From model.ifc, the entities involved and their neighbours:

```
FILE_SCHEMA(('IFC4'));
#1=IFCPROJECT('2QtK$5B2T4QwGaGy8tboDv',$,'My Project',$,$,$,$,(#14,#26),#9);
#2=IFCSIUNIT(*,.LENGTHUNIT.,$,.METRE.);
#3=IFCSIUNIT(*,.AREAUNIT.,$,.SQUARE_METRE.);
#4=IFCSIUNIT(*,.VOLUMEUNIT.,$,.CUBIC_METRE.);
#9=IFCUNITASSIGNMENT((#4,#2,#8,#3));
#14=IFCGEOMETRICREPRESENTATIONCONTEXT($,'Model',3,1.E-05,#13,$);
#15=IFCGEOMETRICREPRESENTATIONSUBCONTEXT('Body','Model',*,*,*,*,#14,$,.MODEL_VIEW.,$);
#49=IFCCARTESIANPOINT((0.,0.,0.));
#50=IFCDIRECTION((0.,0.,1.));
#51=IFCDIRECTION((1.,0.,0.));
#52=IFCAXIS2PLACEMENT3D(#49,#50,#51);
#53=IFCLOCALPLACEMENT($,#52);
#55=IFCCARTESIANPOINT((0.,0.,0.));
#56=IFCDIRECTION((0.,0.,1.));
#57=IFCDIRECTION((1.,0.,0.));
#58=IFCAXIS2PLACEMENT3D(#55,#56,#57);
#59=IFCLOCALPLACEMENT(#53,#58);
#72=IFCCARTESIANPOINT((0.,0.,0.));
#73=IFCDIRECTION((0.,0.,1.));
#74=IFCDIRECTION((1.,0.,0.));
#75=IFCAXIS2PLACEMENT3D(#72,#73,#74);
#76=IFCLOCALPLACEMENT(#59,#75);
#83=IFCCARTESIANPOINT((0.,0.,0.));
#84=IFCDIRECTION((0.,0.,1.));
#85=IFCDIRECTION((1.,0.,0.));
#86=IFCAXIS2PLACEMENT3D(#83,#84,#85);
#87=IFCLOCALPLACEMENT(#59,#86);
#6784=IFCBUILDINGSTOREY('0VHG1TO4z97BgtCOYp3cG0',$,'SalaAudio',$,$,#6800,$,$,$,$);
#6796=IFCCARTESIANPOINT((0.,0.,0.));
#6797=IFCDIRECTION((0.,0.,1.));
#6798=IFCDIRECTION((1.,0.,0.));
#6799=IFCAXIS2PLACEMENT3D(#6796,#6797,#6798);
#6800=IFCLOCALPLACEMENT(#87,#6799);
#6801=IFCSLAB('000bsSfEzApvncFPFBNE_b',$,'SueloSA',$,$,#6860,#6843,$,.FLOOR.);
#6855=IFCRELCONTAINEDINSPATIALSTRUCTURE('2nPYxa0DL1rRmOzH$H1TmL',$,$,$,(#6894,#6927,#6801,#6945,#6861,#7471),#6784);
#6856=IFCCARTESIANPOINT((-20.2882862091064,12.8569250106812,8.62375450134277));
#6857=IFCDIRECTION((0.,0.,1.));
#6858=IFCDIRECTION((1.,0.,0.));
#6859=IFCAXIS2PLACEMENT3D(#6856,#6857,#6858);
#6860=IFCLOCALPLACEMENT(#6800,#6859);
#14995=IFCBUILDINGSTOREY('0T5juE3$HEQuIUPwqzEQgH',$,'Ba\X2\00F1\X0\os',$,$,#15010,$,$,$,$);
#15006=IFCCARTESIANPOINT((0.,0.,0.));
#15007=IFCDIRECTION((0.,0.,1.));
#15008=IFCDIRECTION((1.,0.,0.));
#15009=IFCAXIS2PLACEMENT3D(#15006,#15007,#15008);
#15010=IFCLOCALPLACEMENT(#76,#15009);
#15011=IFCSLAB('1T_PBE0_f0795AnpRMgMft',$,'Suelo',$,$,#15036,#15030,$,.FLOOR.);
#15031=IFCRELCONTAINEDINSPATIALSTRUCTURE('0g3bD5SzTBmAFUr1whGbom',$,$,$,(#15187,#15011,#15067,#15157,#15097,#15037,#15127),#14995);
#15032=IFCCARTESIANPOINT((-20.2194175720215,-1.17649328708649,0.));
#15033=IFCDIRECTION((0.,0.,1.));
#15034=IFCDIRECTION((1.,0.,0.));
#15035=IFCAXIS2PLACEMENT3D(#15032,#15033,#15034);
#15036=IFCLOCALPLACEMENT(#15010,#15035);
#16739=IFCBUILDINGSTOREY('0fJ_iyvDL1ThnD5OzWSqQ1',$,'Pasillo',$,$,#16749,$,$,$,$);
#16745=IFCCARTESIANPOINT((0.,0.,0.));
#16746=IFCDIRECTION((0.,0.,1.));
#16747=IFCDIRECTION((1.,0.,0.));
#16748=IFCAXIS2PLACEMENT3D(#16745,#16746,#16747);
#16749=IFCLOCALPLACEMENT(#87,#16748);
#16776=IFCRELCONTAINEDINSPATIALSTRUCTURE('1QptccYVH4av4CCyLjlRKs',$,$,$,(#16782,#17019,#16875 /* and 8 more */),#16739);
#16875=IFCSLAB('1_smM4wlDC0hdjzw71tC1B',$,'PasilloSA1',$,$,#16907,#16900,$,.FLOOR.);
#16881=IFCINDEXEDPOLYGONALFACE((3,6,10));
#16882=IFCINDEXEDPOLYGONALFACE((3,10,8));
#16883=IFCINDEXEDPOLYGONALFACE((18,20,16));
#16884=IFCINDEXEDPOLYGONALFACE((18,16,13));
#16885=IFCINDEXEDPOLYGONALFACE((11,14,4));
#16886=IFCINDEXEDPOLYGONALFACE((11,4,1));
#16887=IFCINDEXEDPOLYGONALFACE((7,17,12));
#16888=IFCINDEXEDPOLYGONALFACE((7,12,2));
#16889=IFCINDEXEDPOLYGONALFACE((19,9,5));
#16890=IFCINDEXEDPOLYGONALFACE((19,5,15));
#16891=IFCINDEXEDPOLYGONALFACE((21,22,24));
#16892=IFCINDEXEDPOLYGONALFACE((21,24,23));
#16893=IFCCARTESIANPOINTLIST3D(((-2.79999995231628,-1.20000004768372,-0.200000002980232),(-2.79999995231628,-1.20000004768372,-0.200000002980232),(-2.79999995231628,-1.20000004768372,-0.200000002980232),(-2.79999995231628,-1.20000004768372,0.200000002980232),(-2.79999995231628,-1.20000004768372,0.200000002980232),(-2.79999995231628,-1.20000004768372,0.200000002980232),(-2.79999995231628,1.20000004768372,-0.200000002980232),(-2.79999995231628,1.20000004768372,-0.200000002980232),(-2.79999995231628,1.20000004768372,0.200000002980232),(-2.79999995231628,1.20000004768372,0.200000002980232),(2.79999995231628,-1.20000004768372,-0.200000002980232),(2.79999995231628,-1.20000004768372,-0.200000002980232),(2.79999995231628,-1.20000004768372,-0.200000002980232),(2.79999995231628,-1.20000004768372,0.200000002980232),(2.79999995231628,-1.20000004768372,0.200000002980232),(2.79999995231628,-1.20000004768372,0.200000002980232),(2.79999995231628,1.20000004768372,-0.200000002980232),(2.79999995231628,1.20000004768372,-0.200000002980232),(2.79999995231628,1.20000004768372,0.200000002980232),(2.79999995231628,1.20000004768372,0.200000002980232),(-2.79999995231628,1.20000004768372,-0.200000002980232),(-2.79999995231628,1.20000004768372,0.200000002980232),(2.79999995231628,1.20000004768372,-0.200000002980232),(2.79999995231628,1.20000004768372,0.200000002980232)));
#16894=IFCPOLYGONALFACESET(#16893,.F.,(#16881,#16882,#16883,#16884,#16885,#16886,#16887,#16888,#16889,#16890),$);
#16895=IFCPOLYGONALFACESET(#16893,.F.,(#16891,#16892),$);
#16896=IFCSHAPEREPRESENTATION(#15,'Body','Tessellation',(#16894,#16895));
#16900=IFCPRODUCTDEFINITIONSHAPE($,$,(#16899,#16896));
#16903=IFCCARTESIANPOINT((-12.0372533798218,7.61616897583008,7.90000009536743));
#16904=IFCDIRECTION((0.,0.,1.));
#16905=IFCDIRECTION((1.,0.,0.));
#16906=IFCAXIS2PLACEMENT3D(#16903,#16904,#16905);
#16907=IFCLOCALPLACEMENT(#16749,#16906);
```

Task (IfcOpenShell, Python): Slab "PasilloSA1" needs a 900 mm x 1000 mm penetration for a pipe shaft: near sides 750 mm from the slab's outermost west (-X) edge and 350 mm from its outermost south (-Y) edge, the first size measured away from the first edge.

```python
import numpy as np
import ifcopenshell
import ifcopenshell.api.feature
import ifcopenshell.api.geometry
import ifcopenshell.api.root
import ifcopenshell.geom
import ifcopenshell.util.placement
import ifcopenshell.util.representation
import ifcopenshell.util.shape
import ifcopenshell.util.unit

model = ifcopenshell.open("model.ifc")
unit_scale = ifcopenshell.util.unit.calculate_unit_scale(model)
settings = ifcopenshell.geom.settings()


def volume(element):
    """Net volume in cubic metres, openings subtracted."""
    shape = ifcopenshell.geom.create_shape(settings, element)
    return ifcopenshell.util.shape.get_volume(shape.geometry)


slab = model.by_id(16875)
before = volume(slab)

# Extent in the slab's own axes, in metres. The edges named are its -X and -Y sides.
slab_shape = ifcopenshell.geom.create_shape(settings, slab)
vertices = ifcopenshell.util.shape.get_vertices(slab_shape.geometry)
x_min, y_min, bottom = vertices.min(axis=0)
top = vertices[:, 2].max()

opening = ifcopenshell.api.root.create_entity(model, ifc_class="IfcOpeningElement", name="Pipe shaft opening", predefined_type="OPENING")
context = ifcopenshell.util.representation.get_context(model, "Model", "Body", "MODEL_VIEW")
width, depth = 0.9, 1
outline = [(0.0, 0.0), (width, 0.0), (width, depth), (0.0, depth), (0.0, 0.0)]
# Overshoot both faces by 50 mm so the cut is clean.
shape = ifcopenshell.api.geometry.add_slab_representation(
    model, context=context, depth=top - bottom + 0.1, polyline=outline
)
ifcopenshell.api.geometry.assign_representation(model, product=opening, representation=shape)

matrix = ifcopenshell.util.placement.get_local_placement(slab.ObjectPlacement)
matrix[:, 3] = matrix @ np.append(np.array([x_min + 0.75, y_min + 0.35, bottom - 0.05]) / unit_scale, 1.0)
ifcopenshell.api.geometry.edit_object_placement(model, product=opening, matrix=matrix, is_si=False)
ifcopenshell.api.feature.add_feature(model, feature=opening, element=slab)

after = volume(slab)

print(f"slab volume {before:.3f} -> {after:.3f} m3")

model.write("model_updated.ifc")
```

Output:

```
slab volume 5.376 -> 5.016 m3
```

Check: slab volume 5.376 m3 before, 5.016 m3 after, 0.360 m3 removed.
